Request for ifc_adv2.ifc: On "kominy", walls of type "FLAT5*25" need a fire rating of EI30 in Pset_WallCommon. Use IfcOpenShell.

First a look at what the model holds.

```python
import ifcopenshell
import ifcopenshell.util.element

model = ifcopenshell.open("ifc_adv2.ifc")
print(model.schema)
storey = next(s for s in model.by_type("IfcBuildingStorey") if s.Name == "kominy")
walls = [e for e in ifcopenshell.util.element.get_decomposition(storey) if e.is_a("IfcWall")]
seen = {}
for e in walls:
    element_type = ifcopenshell.util.element.get_type(e)
    key = (element_type.Name if element_type != e and element_type else None, ifcopenshell.util.element.get_pset(e, "Pset_WallCommon", "FireRating"))
    seen[key] = seen.get(key, 0) + 1
for (name, value), count in sorted(seen.items(), key=str):
    print(count, "x", name, "|", value)
```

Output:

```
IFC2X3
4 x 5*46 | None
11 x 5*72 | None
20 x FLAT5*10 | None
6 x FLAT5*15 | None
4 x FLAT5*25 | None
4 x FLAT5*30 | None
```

```python
import ifcopenshell
import ifcopenshell.api.pset
import ifcopenshell.util.element

model = ifcopenshell.open("ifc_adv2.ifc")

storey = next(s for s in model.by_type("IfcBuildingStorey") if s.Name == "kominy")
walls = [e for e in ifcopenshell.util.element.get_decomposition(storey) if e.is_a("IfcWall")]

count = 0
for e in walls:
    element_type = ifcopenshell.util.element.get_type(e)
    if element_type in (None, e) or element_type.Name != "FLAT5*25":
        continue
    # add_pset returns the element's existing set when there is one.
    pset = ifcopenshell.api.pset.add_pset(model, product=e, name="Pset_WallCommon")
    ifcopenshell.api.pset.edit_pset(model, pset=pset, properties={"FireRating": "EI30"})
    count += 1

print(count, "walls updated")

model.write("ifc_adv2_updated.ifc")
```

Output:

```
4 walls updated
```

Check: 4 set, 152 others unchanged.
